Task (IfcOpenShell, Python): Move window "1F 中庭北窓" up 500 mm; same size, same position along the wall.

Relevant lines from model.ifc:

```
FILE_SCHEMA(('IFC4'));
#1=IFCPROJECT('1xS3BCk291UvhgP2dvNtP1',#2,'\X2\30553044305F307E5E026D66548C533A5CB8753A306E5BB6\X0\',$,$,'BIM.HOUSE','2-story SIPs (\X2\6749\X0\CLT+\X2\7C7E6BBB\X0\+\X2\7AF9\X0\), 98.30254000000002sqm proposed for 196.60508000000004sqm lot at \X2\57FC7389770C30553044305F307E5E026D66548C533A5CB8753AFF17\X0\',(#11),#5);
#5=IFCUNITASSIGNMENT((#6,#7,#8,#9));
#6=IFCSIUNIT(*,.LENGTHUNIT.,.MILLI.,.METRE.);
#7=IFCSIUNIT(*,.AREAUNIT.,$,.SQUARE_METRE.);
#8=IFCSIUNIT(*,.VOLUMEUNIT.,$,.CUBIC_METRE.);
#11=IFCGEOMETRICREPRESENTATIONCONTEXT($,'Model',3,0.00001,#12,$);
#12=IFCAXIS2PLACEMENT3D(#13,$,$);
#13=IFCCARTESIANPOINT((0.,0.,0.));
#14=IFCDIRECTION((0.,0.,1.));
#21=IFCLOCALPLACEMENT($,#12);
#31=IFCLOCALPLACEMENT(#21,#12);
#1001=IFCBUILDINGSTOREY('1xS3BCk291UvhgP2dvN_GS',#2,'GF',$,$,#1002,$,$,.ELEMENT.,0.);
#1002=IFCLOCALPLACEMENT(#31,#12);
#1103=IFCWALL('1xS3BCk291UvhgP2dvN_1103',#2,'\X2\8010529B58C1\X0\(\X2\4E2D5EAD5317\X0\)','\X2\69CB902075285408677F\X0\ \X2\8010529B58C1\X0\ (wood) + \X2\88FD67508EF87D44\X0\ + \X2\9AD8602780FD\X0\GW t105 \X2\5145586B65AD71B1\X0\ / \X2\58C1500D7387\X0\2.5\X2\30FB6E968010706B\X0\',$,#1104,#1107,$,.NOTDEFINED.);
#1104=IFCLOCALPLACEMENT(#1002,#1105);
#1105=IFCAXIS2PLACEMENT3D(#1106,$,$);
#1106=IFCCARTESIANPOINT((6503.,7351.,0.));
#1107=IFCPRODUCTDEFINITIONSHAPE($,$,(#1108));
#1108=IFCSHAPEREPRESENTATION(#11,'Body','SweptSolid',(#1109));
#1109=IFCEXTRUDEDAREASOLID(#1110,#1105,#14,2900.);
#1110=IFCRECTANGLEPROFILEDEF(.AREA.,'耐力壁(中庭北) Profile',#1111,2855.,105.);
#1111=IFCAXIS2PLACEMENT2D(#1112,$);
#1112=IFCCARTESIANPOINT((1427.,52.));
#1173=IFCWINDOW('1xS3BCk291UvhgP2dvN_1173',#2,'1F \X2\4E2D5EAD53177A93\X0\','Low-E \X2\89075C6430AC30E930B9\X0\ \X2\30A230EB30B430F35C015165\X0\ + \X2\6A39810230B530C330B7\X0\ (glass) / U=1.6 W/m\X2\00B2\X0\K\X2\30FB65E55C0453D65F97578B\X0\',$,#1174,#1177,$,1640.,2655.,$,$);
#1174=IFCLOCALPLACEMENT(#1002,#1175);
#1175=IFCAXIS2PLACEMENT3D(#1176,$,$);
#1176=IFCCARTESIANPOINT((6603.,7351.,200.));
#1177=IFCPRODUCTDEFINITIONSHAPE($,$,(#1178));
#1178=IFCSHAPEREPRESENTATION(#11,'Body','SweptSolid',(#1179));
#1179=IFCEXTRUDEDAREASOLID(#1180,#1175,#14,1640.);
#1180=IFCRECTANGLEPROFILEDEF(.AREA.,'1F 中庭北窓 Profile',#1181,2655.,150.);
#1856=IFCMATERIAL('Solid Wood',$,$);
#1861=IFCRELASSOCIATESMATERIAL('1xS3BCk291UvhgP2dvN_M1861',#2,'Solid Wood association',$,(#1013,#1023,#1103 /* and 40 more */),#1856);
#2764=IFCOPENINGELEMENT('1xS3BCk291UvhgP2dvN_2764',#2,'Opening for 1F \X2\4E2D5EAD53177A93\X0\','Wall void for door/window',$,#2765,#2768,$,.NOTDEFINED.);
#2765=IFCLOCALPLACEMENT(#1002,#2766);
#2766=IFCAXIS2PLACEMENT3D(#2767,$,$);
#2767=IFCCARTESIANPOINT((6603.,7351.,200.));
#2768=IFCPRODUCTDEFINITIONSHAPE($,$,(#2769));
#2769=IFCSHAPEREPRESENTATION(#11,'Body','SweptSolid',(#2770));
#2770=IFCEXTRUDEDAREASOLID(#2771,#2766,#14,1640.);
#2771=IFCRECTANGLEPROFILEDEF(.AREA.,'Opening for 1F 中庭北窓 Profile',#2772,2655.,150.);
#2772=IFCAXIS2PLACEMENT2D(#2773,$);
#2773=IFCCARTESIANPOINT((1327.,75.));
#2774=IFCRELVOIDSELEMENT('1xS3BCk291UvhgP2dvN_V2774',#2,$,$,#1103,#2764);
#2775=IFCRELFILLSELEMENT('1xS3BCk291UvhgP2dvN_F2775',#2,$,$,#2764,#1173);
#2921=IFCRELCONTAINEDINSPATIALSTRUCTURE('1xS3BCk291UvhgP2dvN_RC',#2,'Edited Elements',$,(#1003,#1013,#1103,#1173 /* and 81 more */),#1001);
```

```python
import numpy as np
import ifcopenshell
import ifcopenshell.api.geometry
import ifcopenshell.util.placement
import ifcopenshell.util.unit

model = ifcopenshell.open("model.ifc")
unit_scale = ifcopenshell.util.unit.calculate_unit_scale(model)

window = model.by_guid("1xS3BCk291UvhgP2dvN_1173")
opening = window.FillsVoids[0].RelatingOpeningElement
dz = 500.0

shift = np.array([0.0, 0.0, dz])
# The window is not placed relative to its opening, so move both.
for product in (opening, window):
    matrix = ifcopenshell.util.placement.get_local_placement(product.ObjectPlacement)
    matrix[:3, 3] += shift
    ifcopenshell.api.geometry.edit_object_placement(model, product=product, matrix=matrix, is_si=False)

print(f"moved by {dz * unit_scale:+.3f} m")

model.write("model_v2.ifc")
```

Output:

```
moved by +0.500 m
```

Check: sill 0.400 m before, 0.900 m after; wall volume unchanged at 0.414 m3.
